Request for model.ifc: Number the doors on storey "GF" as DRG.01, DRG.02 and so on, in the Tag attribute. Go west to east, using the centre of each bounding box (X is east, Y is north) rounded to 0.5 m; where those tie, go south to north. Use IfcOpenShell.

First a look at what the model holds.

```python
import ifcopenshell
import ifcopenshell.util.element
import ifcopenshell.util.placement

model = ifcopenshell.open("model.ifc")
print(model.schema)
storey = next(s for s in model.by_type("IfcBuildingStorey") if s.Name == "GF")
doors = [e for e in ifcopenshell.util.element.get_decomposition(storey) if e.is_a("IfcDoor")]
for e in sorted(doors, key=lambda e: e.id()):
    origin = ifcopenshell.util.placement.get_local_placement(e.ObjectPlacement)[:3, 3]
    print(e.id(), e.Tag, e.Name, origin.round(2) + 0.0, sep=" | ")
```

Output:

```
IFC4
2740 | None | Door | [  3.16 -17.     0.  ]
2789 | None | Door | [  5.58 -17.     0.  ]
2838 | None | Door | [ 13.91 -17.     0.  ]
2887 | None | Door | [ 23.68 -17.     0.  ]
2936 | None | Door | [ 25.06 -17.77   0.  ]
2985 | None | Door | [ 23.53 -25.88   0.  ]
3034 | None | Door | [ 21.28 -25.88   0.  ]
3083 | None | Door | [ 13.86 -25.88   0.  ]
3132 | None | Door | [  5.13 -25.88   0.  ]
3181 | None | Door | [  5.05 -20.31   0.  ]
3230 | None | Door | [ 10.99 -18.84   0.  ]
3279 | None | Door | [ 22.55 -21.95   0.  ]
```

```python
import ifcopenshell
import ifcopenshell.geom
import ifcopenshell.util.element
import ifcopenshell.util.shape

model = ifcopenshell.open("model.ifc")
settings = ifcopenshell.geom.settings()
settings.set("use-world-coords", True)


def centre(element):
    shape = ifcopenshell.geom.create_shape(settings, element)
    return ifcopenshell.util.shape.get_bbox_centroid(shape.geometry)


storey = next(s for s in model.by_type("IfcBuildingStorey") if s.Name == "GF")
doors = [e for e in ifcopenshell.util.element.get_decomposition(storey) if e.is_a("IfcDoor")]

# Insertion points can sit at a corner or the storey origin, so sort by the geometry (in metres).
centres = {e: centre(e) for e in doors}
doors.sort(key=lambda e: (round(centres[e][0] / 0.5), centres[e][1]))

for i, e in enumerate(doors, start=1):
    number = f"DRG.{i:02d}"
    e.Tag = number
    print(e.id(), number)

model.write("model_v2.ifc")
```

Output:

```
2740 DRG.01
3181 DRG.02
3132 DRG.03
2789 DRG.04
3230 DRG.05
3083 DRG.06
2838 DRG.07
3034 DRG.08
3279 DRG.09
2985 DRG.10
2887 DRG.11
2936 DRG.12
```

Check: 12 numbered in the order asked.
